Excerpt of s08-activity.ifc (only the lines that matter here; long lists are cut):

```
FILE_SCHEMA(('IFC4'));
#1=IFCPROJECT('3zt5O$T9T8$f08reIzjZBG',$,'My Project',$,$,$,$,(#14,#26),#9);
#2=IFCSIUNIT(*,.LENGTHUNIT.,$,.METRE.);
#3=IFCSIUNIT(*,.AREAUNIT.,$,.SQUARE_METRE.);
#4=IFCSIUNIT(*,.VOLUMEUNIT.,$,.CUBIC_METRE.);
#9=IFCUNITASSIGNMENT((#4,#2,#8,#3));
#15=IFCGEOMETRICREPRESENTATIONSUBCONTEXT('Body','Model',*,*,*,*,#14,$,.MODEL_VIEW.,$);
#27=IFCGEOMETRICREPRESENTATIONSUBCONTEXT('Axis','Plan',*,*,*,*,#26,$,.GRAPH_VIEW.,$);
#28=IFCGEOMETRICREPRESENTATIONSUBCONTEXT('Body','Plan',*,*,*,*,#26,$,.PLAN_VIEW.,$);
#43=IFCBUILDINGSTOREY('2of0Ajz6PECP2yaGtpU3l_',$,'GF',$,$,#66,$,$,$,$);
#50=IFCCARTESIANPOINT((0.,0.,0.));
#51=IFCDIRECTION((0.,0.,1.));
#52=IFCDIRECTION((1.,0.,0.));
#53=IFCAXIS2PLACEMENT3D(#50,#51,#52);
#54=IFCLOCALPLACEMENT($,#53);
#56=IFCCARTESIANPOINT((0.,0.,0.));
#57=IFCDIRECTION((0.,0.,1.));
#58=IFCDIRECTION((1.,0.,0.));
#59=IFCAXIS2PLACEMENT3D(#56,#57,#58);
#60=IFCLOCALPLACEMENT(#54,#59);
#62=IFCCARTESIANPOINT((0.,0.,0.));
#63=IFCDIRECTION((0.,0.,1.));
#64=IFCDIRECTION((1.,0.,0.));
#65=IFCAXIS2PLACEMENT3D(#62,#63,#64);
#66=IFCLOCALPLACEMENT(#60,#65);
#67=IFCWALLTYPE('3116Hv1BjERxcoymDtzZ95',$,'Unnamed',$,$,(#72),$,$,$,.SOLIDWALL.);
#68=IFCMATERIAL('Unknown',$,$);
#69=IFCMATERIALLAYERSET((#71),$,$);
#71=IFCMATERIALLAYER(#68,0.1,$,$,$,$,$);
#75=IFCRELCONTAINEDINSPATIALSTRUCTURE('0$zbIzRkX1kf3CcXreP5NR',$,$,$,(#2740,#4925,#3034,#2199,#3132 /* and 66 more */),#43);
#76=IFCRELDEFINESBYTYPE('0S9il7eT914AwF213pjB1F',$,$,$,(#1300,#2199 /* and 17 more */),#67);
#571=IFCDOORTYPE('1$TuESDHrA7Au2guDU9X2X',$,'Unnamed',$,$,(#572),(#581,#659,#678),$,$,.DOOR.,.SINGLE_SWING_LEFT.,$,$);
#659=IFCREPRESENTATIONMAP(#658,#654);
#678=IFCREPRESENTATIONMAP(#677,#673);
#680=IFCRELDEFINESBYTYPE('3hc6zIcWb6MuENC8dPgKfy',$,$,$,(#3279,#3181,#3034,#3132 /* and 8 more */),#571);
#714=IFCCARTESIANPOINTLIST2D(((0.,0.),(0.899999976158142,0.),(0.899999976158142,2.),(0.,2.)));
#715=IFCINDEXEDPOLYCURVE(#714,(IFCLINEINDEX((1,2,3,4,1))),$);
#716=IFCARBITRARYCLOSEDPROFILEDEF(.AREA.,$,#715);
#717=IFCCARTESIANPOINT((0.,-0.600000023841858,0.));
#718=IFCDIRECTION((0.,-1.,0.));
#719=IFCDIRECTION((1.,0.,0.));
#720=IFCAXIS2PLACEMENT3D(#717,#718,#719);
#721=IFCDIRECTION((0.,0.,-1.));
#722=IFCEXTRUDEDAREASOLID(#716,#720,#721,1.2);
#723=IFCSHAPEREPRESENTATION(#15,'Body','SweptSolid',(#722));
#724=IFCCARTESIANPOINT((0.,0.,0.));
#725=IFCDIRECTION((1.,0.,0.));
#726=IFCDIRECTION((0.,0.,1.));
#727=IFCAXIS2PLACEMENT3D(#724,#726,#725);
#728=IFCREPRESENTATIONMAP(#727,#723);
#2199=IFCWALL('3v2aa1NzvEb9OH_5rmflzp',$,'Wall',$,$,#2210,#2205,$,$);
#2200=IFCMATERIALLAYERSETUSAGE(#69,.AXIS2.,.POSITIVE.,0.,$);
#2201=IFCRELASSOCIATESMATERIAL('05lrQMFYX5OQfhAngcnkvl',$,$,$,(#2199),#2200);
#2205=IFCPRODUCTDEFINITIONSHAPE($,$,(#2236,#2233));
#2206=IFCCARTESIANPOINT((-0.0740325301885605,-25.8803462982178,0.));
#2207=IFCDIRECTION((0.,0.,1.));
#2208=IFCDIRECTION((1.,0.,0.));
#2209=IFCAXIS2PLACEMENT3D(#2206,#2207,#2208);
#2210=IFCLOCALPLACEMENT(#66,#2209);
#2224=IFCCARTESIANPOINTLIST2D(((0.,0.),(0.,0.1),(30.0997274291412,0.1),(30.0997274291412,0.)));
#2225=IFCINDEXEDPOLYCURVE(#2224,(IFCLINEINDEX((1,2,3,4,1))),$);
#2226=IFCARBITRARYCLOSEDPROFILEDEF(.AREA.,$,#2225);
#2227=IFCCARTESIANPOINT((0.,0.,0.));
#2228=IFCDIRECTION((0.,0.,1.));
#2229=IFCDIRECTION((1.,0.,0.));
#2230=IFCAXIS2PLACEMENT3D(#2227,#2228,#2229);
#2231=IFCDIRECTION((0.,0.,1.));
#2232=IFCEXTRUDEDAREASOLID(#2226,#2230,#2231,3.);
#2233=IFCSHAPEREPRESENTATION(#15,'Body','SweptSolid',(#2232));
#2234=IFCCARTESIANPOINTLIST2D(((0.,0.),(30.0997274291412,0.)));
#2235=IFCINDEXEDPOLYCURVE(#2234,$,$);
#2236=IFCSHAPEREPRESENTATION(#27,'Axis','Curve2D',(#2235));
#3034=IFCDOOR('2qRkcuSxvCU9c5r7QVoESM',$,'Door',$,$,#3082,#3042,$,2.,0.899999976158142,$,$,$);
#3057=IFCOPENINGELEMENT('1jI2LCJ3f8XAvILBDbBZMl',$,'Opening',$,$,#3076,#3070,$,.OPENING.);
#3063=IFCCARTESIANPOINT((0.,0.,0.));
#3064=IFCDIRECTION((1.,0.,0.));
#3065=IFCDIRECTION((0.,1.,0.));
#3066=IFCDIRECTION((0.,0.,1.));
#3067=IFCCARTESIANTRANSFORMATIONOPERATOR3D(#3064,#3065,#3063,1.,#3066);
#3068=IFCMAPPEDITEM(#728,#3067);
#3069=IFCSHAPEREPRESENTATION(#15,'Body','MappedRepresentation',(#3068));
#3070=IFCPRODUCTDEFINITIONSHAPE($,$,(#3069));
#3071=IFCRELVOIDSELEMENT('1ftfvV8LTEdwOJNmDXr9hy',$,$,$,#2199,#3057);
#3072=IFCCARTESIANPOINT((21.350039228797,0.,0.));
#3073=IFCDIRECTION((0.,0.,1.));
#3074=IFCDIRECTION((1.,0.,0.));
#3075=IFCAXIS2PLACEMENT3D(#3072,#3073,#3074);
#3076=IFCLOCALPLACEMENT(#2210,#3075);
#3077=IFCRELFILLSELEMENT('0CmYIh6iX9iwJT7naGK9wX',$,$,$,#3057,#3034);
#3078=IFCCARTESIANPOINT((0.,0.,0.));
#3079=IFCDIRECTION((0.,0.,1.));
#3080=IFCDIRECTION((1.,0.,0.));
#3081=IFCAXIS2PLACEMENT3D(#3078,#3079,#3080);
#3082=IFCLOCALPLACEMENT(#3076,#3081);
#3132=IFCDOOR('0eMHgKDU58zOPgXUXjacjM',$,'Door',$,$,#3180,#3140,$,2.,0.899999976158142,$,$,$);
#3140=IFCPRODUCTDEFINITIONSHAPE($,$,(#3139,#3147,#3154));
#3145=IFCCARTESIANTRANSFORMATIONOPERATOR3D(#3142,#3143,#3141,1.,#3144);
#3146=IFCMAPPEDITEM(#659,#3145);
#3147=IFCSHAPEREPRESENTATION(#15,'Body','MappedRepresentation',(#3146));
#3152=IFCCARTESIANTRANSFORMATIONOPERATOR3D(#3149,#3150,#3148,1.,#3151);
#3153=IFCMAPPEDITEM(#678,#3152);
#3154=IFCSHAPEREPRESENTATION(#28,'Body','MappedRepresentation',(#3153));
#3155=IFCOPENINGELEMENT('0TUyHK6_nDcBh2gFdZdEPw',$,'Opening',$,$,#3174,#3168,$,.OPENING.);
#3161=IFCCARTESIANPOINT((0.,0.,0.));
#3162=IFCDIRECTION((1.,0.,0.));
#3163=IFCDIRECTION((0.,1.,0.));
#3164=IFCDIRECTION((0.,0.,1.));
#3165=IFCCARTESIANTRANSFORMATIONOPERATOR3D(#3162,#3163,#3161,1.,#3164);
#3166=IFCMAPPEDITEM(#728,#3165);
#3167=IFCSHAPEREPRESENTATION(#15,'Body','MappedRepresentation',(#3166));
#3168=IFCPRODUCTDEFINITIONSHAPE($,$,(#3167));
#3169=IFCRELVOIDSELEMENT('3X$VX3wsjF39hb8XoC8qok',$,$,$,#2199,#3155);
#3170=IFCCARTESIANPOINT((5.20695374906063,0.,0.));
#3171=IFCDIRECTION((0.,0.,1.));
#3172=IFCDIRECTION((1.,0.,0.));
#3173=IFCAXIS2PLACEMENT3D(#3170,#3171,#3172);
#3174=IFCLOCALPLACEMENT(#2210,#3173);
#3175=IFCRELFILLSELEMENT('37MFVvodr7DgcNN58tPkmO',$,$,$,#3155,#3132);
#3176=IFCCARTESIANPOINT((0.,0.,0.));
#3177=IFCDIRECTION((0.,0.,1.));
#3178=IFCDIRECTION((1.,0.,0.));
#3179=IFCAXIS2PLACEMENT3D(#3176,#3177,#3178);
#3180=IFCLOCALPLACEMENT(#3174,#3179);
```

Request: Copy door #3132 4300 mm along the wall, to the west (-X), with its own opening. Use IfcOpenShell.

```python
import ifcopenshell
import ifcopenshell.api.feature
import ifcopenshell.api.geometry
import ifcopenshell.api.root
import ifcopenshell.geom
import ifcopenshell.util.element
import ifcopenshell.util.placement
import ifcopenshell.util.shape

model = ifcopenshell.open("s08-activity.ifc")
settings = ifcopenshell.geom.settings()


def volume(element):
    """Net volume in cubic metres, openings subtracted."""
    shape = ifcopenshell.geom.create_shape(settings, element)
    return ifcopenshell.util.shape.get_volume(shape.geometry)


door = model.by_id(3132)
opening = door.FillsVoids[0].RelatingOpeningElement
wall = opening.VoidsElements[0].RelatingBuildingElement
before = volume(wall)
shift = ifcopenshell.util.placement.get_local_placement(wall.ObjectPlacement)[:3, 0] * -4.3

# copy_class copies the void relationship, type, container and properties, but no geometry.
new_opening = ifcopenshell.api.root.copy_class(model, product=opening)
new_opening.Representation = ifcopenshell.util.element.copy_deep(
    model, opening.Representation, exclude=["IfcGeometricRepresentationContext", "IfcRepresentationMap"]
)
new_door = ifcopenshell.api.root.copy_class(model, product=door)
new_door.Representation = ifcopenshell.util.element.copy_deep(
    model, door.Representation, exclude=["IfcGeometricRepresentationContext", "IfcRepresentationMap"]
)
ifcopenshell.api.feature.add_filling(model, opening=new_opening, element=new_door)

for old, new in ((opening, new_opening), (door, new_door)):
    matrix = ifcopenshell.util.placement.get_local_placement(old.ObjectPlacement)
    matrix[:3, 3] += shift
    ifcopenshell.api.geometry.edit_object_placement(model, product=new, matrix=matrix, is_si=False)

after = volume(wall)

print(f"wall volume {before:.3f} -> {after:.3f} m3")

model.write("s08-activity_edited.ifc")
```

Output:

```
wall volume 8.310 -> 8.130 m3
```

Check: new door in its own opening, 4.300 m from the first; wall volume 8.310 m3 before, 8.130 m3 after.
